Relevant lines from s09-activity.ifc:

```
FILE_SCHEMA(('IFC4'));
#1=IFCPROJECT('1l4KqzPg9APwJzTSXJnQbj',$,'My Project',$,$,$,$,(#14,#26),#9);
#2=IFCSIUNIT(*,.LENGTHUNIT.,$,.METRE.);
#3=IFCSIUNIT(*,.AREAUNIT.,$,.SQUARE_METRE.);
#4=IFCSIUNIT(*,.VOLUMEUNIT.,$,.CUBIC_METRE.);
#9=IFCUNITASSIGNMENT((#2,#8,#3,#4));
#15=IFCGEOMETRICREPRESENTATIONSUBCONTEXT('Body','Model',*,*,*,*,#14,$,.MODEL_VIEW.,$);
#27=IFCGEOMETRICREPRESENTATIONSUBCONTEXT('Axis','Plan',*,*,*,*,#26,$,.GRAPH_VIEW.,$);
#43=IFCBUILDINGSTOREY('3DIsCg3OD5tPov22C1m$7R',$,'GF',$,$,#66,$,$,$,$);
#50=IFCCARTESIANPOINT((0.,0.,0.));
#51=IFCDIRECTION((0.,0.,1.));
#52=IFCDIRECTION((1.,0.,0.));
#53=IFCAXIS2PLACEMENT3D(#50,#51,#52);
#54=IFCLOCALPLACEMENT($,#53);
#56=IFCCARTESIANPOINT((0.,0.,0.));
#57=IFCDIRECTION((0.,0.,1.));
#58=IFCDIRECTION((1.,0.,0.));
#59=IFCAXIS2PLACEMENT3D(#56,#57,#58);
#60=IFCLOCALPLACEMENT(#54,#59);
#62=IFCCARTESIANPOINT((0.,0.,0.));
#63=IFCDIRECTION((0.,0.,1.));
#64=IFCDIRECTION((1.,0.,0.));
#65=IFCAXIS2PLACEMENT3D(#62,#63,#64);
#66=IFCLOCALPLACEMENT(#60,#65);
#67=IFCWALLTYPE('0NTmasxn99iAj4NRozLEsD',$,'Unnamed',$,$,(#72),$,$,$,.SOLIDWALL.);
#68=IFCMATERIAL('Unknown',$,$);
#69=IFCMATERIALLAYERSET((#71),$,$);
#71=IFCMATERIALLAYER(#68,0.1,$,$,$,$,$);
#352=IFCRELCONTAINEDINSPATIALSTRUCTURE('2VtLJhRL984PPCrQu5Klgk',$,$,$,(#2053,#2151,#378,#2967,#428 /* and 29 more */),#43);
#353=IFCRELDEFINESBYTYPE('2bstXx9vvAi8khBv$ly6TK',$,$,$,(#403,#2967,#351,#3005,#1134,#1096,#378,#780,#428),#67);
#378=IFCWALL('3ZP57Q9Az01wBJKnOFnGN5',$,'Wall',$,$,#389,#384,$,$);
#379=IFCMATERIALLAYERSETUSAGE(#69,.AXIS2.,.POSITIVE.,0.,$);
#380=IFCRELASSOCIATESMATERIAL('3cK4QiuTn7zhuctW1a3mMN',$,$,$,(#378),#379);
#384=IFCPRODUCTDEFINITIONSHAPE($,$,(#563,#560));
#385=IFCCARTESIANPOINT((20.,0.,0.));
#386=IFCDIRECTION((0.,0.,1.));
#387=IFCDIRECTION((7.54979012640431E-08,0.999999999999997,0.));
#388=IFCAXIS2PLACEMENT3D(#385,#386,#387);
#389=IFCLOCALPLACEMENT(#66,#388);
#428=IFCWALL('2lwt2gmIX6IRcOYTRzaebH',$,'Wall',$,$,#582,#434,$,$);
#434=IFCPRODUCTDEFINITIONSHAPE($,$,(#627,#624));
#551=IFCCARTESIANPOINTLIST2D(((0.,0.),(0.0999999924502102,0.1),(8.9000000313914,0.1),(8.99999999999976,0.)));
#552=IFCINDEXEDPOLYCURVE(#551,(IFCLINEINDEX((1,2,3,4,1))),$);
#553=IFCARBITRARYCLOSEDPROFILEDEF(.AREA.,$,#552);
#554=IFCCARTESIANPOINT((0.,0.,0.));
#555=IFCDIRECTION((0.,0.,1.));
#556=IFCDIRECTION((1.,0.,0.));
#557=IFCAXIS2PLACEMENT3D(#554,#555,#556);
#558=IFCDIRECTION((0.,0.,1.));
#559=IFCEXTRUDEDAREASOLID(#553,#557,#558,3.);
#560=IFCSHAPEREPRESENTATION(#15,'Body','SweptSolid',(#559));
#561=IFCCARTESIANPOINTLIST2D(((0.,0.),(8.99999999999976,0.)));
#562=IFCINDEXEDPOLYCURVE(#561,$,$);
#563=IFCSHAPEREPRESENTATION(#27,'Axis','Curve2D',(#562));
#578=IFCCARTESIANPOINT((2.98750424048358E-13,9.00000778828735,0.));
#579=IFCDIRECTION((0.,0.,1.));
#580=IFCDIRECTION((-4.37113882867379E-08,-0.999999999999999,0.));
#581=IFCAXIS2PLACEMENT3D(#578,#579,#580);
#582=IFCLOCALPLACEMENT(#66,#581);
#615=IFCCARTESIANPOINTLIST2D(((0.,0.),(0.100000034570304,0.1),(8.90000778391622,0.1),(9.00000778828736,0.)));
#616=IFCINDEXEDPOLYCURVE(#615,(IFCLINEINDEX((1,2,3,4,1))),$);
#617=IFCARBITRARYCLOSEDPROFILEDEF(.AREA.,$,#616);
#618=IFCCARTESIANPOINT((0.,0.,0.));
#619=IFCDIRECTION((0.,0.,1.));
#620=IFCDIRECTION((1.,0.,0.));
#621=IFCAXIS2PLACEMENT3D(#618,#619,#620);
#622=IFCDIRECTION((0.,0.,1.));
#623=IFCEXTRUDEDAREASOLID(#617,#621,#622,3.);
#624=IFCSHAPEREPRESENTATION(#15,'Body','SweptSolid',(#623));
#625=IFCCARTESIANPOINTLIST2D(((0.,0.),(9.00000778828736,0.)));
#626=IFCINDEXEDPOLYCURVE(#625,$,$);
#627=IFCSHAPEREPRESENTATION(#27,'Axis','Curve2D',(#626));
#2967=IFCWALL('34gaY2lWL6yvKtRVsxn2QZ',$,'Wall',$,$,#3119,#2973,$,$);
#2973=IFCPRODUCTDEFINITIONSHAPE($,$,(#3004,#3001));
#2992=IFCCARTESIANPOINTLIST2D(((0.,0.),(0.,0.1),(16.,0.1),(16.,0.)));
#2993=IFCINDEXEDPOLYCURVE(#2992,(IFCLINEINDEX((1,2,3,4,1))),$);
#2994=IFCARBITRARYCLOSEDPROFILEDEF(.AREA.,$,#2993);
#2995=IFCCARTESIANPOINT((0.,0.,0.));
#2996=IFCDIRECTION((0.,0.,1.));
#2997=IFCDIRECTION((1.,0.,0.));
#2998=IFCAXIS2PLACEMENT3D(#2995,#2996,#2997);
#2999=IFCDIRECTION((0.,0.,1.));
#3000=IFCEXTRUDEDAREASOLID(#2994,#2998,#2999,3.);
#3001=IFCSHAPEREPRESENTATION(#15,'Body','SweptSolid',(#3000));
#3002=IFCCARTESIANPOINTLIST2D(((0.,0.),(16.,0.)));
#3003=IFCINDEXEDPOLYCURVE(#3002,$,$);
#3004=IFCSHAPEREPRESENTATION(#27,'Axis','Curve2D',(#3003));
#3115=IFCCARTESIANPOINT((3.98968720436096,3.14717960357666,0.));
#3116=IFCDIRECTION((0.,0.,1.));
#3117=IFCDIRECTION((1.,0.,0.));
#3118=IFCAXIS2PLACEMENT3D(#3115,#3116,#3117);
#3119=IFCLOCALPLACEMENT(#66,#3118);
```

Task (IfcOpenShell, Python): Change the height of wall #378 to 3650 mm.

```python
import ifcopenshell
import ifcopenshell.geom
import ifcopenshell.util.representation
import ifcopenshell.util.shape

model = ifcopenshell.open("s09-activity.ifc")
settings = ifcopenshell.geom.settings()


def volume(element):
    """Net volume in cubic metres, openings subtracted."""
    shape = ifcopenshell.geom.create_shape(settings, element)
    return ifcopenshell.util.shape.get_volume(shape.geometry)


wall = model.by_guid("3ZP57Q9Az01wBJKnOFnGN5")
before = volume(wall)

body = ifcopenshell.util.representation.get_representation(wall, "Model", "Body")
solid = body.Items[0]
old_height = solid.Depth
solid.Depth = 3.65
after = volume(wall)

print(f"height {old_height:g} -> {solid.Depth:g}, volume {before:.3f} -> {after:.3f} m3")

model.write("s09-activity_edited.ifc")
```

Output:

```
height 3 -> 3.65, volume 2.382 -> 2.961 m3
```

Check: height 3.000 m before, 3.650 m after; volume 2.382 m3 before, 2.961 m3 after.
